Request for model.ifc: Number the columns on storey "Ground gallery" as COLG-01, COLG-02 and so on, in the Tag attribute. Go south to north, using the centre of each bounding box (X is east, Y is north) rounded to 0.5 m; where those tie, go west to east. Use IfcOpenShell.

First a look at what the model holds.

```python
import ifcopenshell
import ifcopenshell.util.element
import ifcopenshell.util.placement

model = ifcopenshell.open("model.ifc")
print(model.schema)
storey = next(s for s in model.by_type("IfcBuildingStorey") if s.Name == "Ground gallery")
columns = [e for e in ifcopenshell.util.element.get_decomposition(storey) if e.is_a("IfcColumn")]
for e in sorted(columns, key=lambda e: e.id()):
    origin = ifcopenshell.util.placement.get_local_placement(e.ObjectPlacement)[:3, 3]
    print(e.id(), e.Tag, e.Name, origin.round(2) + 0.0, sep=" | ")
```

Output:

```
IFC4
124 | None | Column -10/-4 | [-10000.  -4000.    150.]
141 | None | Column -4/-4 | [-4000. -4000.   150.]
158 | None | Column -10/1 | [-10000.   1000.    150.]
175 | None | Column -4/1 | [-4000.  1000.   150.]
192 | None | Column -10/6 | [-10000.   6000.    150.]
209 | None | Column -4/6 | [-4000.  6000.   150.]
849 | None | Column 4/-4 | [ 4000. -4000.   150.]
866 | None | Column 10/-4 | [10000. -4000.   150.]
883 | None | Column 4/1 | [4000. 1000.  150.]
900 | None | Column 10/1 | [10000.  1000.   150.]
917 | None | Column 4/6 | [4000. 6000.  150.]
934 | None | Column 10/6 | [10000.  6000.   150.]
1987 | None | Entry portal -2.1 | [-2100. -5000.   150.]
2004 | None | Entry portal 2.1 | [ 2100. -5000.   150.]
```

```python
import ifcopenshell
import ifcopenshell.geom
import ifcopenshell.util.element
import ifcopenshell.util.shape

model = ifcopenshell.open("model.ifc")
settings = ifcopenshell.geom.settings()
settings.set("use-world-coords", True)


def centre(element):
    shape = ifcopenshell.geom.create_shape(settings, element)
    return ifcopenshell.util.shape.get_bbox_centroid(shape.geometry)


storey = next(s for s in model.by_type("IfcBuildingStorey") if s.Name == "Ground gallery")
columns = [e for e in ifcopenshell.util.element.get_decomposition(storey) if e.is_a("IfcColumn")]

# Insertion points can sit at a corner or the storey origin, so sort by the geometry (in metres).
centres = {e: centre(e) for e in columns}
columns.sort(key=lambda e: (round(centres[e][1] / 0.5), centres[e][0]))

for i, e in enumerate(columns, start=1):
    number = f"COLG-{i:02d}"
    e.Tag = number
    print(e.id(), number)

model.write("model_edited.ifc")
```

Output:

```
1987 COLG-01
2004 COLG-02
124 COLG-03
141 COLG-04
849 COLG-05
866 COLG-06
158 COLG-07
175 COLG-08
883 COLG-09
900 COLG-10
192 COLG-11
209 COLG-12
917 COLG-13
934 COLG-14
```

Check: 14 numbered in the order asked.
